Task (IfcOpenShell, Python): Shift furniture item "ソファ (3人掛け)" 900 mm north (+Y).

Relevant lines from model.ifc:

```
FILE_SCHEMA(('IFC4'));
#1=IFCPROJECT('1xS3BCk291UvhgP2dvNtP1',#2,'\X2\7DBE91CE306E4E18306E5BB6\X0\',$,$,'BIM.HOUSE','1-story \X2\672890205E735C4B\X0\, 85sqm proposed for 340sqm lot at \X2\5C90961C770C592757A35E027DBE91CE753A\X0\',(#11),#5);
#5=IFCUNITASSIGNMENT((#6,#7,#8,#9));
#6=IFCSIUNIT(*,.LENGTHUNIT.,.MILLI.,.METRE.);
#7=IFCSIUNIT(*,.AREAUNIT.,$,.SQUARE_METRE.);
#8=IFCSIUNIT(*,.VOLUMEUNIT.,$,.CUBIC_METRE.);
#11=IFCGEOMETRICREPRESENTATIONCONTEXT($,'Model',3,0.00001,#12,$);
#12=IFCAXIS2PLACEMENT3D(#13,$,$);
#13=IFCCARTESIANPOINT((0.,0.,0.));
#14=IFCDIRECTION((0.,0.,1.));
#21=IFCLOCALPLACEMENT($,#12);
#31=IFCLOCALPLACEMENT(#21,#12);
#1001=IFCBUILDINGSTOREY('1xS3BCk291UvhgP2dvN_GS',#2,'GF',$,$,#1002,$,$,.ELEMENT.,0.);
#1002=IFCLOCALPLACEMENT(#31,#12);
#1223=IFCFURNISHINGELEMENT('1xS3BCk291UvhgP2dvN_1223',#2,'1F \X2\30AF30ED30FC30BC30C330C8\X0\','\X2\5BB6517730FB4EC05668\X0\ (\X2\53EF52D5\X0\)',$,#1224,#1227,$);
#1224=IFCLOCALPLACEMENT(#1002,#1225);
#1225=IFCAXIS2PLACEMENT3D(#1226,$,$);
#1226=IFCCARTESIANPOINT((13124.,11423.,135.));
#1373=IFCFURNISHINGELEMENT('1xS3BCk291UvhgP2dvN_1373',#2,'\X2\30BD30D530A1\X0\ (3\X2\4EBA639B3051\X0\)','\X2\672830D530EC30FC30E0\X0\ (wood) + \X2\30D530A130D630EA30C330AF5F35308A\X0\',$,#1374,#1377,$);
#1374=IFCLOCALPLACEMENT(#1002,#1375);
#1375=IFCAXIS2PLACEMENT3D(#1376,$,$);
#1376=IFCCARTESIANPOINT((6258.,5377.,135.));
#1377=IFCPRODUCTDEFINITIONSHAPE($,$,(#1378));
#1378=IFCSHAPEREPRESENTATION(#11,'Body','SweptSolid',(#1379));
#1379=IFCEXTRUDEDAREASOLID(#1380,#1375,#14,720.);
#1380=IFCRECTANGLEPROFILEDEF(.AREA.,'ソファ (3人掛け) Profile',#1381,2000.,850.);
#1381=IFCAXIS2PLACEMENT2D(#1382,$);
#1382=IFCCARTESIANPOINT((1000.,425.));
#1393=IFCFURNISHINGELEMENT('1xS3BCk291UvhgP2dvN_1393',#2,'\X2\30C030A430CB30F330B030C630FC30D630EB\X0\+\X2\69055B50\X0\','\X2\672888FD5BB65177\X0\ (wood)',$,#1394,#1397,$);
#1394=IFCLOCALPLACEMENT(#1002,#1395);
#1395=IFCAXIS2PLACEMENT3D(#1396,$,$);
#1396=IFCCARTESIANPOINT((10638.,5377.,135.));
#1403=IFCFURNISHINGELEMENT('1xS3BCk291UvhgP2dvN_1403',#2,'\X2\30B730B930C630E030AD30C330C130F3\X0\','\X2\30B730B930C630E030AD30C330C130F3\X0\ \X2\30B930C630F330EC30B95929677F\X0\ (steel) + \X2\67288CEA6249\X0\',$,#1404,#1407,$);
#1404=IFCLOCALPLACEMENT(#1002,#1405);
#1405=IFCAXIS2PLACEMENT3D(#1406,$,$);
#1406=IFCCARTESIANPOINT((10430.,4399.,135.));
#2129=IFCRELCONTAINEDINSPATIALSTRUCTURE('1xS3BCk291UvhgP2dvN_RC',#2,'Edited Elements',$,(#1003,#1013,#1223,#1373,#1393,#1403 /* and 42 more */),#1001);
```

```python
import ifcopenshell
import ifcopenshell.api.geometry
import ifcopenshell.util.placement

model = ifcopenshell.open("model.ifc")

item = model.by_guid("1xS3BCk291UvhgP2dvN_1373")
matrix = ifcopenshell.util.placement.get_local_placement(item.ObjectPlacement)
matrix[1, 3] += 900.0
ifcopenshell.api.geometry.edit_object_placement(model, product=item, matrix=matrix, is_si=False)

print(ifcopenshell.util.placement.get_local_placement(item.ObjectPlacement).round(3) + 0.0)

model.write("model-out.ifc")
```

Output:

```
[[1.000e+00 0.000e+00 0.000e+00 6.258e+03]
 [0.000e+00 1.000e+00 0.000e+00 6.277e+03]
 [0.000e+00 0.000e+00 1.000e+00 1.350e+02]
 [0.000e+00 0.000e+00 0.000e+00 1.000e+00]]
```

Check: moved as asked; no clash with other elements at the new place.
